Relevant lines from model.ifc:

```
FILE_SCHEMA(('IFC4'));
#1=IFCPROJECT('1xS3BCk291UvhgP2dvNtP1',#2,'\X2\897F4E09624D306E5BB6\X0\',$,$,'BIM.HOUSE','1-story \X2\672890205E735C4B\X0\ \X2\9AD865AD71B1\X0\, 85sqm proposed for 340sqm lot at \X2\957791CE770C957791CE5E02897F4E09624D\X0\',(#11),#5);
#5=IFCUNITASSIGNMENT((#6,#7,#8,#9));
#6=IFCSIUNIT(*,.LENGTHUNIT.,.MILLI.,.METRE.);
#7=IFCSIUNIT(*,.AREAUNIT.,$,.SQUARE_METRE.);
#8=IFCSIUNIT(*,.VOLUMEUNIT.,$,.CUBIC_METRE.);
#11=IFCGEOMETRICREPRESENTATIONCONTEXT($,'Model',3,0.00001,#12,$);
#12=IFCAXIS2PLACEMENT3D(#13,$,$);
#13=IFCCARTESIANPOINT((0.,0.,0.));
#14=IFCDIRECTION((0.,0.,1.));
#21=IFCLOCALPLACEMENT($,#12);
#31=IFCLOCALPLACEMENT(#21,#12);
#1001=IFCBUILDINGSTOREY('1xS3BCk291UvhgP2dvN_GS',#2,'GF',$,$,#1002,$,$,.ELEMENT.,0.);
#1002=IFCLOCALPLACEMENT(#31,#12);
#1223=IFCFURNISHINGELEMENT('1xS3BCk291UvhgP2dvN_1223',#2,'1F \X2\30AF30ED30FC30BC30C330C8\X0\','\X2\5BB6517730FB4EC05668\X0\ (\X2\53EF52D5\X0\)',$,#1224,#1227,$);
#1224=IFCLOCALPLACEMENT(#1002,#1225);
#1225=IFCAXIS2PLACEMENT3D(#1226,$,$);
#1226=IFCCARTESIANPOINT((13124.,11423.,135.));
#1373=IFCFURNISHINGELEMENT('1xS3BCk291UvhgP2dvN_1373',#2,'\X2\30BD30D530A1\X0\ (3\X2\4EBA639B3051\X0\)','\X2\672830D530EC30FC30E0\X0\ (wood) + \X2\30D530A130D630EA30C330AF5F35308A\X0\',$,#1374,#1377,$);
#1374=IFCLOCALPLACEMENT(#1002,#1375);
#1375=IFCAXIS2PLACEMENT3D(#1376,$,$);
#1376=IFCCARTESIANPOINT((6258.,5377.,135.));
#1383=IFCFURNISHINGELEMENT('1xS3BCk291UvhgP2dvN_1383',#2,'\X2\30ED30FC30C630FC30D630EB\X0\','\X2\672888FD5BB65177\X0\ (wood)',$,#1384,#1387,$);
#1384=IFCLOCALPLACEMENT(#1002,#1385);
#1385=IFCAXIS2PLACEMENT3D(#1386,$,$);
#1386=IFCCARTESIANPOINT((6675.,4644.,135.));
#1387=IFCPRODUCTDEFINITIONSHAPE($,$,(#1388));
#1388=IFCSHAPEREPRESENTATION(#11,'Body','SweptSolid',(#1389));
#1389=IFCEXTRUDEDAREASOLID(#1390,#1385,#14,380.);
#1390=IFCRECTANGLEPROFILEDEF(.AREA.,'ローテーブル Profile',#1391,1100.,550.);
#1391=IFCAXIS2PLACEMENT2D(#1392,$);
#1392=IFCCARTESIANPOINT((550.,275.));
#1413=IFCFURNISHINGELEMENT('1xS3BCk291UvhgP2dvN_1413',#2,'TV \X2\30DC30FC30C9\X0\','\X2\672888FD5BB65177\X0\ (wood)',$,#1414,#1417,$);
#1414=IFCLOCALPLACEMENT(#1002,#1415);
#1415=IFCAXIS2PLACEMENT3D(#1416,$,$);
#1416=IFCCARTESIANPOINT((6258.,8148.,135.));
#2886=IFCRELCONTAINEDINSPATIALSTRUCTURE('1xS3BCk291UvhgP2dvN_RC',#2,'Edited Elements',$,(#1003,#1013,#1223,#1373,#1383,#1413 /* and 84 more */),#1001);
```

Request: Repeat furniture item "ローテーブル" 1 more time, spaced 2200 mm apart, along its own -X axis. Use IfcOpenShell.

```python
import ifcopenshell
import ifcopenshell.api.geometry
import ifcopenshell.api.root
import ifcopenshell.util.element
import ifcopenshell.util.placement
import ifcopenshell.util.unit

model = ifcopenshell.open("model.ifc")
unit_scale = ifcopenshell.util.unit.calculate_unit_scale(model)


def reuse_history(source, copy):
    """copy_class also copies each property set's owner history, people and application; keep the originals."""
    for rel in copy.IsDefinedBy:
        if rel.is_a("IfcRelDefinesByProperties") and (history := rel.RelatingPropertyDefinition.OwnerHistory):
            rel.RelatingPropertyDefinition.OwnerHistory = source.OwnerHistory
            ifcopenshell.util.element.remove_deep2(model, history)


source = model.by_guid("1xS3BCk291UvhgP2dvN_1383")
base = ifcopenshell.util.placement.get_local_placement(source.ObjectPlacement)
step = -base[:3, 0] * 2.2 / unit_scale

for i in range(1, 2):
    copy = ifcopenshell.api.root.copy_class(model, product=source)
    copy.Representation = ifcopenshell.util.element.copy_deep(
        model, source.Representation, exclude=["IfcGeometricRepresentationContext", "IfcRepresentationMap"]
    )
    reuse_history(source, copy)
    matrix = base.copy()
    matrix[:3, 3] += i * step
    print("added at", matrix[:3, 3].round(3) + 0.0)
    ifcopenshell.api.geometry.edit_object_placement(model, product=copy, matrix=matrix, is_si=False)

model.write("model_edited.ifc")
```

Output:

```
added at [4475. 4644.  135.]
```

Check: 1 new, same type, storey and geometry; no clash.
